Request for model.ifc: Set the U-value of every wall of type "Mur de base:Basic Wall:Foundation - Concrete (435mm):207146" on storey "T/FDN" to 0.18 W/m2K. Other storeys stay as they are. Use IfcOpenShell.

First a look at what the model holds.

```python
import ifcopenshell
import ifcopenshell.util.element

model = ifcopenshell.open("model.ifc")
print(model.schema)
storey = next(s for s in model.by_type("IfcBuildingStorey") if s.Name == "T/FDN")
walls = [e for e in ifcopenshell.util.element.get_decomposition(storey) if e.is_a("IfcWall")]
seen = {}
for e in walls:
    element_type = ifcopenshell.util.element.get_type(e)
    key = (element_type.Name if element_type != e and element_type else None, ifcopenshell.util.element.get_pset(e, "Pset_WallCommon", "ThermalTransmittance"))
    seen[key] = seen.get(key, 0) + 1
for (name, value), count in sorted(seen.items(), key=str):
    print(count, "x", name, "|", value)
```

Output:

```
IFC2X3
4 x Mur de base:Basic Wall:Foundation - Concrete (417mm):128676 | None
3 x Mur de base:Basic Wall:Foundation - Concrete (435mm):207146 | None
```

```python
import ifcopenshell
import ifcopenshell.api.pset
import ifcopenshell.util.element

model = ifcopenshell.open("model.ifc")

storey = next(s for s in model.by_type("IfcBuildingStorey") if s.Name == "T/FDN")
walls = [e for e in ifcopenshell.util.element.get_decomposition(storey) if e.is_a("IfcWall")]

count = 0
for e in walls:
    element_type = ifcopenshell.util.element.get_type(e)
    if element_type in (None, e) or element_type.Name != "Mur de base:Basic Wall:Foundation - Concrete (435mm):207146":
        continue
    # add_pset returns the element's existing set when there is one.
    pset = ifcopenshell.api.pset.add_pset(model, product=e, name="Pset_WallCommon")
    ifcopenshell.api.pset.edit_pset(model, pset=pset, properties={"ThermalTransmittance": 0.18})
    count += 1

print(count, "walls updated")

model.write("model_v2.ifc")
```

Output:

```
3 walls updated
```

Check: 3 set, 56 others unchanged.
